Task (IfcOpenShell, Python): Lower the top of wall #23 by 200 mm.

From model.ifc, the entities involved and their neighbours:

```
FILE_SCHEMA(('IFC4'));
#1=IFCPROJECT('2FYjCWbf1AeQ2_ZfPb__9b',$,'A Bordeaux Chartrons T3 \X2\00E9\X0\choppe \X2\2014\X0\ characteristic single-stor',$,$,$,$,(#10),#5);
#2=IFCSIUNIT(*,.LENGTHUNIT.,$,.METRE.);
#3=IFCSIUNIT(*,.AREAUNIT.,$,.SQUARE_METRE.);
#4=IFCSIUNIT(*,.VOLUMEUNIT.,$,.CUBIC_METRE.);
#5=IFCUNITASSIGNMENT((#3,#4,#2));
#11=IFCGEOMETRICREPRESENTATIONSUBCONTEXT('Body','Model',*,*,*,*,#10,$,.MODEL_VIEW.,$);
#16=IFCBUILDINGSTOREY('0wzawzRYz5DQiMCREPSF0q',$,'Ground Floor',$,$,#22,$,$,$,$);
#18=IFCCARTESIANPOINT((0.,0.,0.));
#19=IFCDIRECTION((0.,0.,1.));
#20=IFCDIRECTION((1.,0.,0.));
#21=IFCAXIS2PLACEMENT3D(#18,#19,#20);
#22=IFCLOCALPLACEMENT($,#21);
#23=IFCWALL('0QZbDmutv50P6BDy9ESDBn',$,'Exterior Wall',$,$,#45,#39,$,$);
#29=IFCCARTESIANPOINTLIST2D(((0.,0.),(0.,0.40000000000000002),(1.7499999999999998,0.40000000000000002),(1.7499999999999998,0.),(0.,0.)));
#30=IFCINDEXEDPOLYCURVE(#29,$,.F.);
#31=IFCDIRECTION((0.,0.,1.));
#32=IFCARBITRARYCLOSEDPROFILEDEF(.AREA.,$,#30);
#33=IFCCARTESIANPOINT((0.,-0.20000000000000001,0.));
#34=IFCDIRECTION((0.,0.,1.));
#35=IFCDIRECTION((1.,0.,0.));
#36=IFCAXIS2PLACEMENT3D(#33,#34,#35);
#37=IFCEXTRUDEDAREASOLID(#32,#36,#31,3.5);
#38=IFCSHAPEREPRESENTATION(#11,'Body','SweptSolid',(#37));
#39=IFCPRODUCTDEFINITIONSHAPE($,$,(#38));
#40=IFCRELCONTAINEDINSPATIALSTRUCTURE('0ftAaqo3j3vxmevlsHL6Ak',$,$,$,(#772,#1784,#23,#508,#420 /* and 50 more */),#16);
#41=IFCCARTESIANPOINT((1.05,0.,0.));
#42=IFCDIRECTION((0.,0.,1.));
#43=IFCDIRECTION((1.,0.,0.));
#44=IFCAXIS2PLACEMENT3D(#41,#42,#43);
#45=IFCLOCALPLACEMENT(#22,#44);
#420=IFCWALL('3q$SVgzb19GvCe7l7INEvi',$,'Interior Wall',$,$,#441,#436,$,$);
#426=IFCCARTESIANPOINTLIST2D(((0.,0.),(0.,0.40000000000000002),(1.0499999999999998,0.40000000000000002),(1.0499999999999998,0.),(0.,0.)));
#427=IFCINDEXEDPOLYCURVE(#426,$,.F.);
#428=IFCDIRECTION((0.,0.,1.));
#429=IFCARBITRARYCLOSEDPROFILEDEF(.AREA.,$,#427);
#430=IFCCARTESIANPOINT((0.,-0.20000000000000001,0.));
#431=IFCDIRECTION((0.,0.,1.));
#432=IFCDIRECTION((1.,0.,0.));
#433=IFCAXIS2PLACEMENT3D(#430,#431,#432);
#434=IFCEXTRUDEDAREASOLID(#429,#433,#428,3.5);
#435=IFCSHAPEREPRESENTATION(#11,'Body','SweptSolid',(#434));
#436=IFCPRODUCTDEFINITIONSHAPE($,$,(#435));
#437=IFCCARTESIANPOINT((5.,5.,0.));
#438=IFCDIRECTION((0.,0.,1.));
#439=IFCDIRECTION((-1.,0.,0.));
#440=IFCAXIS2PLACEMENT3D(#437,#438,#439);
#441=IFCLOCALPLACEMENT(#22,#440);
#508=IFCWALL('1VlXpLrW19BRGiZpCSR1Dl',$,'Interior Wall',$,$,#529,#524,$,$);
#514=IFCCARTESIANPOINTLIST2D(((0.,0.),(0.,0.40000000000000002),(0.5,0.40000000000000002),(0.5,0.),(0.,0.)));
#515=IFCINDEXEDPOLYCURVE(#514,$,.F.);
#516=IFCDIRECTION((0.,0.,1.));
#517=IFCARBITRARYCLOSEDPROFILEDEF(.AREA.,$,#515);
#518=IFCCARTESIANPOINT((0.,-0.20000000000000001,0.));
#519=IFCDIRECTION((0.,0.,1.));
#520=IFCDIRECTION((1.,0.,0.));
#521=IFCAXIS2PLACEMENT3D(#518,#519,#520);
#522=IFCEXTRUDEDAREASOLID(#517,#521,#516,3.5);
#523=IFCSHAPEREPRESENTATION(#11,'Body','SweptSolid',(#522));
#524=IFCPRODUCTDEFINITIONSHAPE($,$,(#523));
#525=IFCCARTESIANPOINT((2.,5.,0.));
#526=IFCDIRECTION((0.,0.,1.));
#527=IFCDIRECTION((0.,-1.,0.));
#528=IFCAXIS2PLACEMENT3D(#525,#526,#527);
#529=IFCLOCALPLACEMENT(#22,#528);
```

```python
import ifcopenshell
import ifcopenshell.geom
import ifcopenshell.util.representation
import ifcopenshell.util.shape
import ifcopenshell.util.unit

model = ifcopenshell.open("model.ifc")
unit_scale = ifcopenshell.util.unit.calculate_unit_scale(model)
settings = ifcopenshell.geom.settings()


def volume(element):
    """Net volume in cubic metres, openings subtracted."""
    shape = ifcopenshell.geom.create_shape(settings, element)
    return ifcopenshell.util.shape.get_volume(shape.geometry)


wall = model.by_guid("0QZbDmutv50P6BDy9ESDBn")
before = volume(wall)

body = ifcopenshell.util.representation.get_representation(wall, "Model", "Body")
solid = body.Items[0]
old_height = solid.Depth
solid.Depth -= 0.2 / unit_scale
after = volume(wall)

print(f"height {old_height:g} -> {solid.Depth:g}, volume {before:.3f} -> {after:.3f} m3")

model.write("model_v2.ifc")
```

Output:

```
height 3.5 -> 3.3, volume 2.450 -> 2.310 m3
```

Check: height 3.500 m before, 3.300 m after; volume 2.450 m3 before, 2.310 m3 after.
